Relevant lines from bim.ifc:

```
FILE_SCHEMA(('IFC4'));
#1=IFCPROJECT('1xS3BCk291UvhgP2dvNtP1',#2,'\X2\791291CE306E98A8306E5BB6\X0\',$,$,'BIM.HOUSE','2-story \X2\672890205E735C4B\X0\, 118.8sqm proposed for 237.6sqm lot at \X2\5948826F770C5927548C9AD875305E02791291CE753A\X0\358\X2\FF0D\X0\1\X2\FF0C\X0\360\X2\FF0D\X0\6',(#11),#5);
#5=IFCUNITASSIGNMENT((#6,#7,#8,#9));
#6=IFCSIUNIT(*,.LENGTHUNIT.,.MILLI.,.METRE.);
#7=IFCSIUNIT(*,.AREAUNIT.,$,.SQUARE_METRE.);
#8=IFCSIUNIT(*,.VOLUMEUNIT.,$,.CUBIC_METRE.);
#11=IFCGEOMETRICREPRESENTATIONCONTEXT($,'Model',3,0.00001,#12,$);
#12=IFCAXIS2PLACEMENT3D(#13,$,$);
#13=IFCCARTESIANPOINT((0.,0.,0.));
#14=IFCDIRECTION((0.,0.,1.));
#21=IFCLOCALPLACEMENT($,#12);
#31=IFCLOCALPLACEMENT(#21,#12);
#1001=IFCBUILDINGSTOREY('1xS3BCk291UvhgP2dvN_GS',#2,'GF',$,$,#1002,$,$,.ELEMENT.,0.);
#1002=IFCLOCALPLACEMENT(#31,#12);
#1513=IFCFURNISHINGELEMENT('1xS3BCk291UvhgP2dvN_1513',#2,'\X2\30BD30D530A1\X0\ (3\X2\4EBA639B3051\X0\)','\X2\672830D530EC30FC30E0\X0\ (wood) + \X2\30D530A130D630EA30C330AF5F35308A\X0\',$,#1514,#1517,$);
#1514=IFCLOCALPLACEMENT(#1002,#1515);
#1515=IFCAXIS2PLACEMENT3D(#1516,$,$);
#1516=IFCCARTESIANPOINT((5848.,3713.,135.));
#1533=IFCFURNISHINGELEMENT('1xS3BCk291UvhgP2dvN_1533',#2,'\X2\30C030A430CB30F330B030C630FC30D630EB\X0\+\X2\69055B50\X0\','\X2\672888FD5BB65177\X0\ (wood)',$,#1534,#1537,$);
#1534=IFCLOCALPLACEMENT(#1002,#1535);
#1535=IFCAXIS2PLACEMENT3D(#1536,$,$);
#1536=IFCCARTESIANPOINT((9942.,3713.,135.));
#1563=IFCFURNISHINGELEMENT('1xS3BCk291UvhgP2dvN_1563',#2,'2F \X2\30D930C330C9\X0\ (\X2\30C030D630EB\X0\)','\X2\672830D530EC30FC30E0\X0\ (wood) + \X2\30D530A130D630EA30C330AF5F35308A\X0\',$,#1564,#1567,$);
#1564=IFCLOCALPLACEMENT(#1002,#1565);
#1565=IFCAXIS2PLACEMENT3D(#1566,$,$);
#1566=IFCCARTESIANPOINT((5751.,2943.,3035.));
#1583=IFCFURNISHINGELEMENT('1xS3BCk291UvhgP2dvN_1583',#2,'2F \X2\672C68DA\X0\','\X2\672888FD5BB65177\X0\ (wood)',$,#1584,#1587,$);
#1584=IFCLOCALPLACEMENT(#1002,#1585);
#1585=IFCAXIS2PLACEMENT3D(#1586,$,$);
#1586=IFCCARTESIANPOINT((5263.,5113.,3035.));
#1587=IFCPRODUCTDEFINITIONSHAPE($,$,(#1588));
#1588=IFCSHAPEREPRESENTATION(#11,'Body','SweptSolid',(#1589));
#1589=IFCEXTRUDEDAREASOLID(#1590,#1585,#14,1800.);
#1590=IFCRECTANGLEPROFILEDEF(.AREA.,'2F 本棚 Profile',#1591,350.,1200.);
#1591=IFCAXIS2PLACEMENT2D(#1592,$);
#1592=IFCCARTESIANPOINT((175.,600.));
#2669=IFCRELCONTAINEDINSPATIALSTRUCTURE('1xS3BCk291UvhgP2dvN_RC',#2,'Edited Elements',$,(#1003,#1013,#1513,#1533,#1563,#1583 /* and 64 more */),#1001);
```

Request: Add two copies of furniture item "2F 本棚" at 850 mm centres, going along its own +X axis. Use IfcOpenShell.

```python
import ifcopenshell
import ifcopenshell.api.geometry
import ifcopenshell.api.root
import ifcopenshell.util.element
import ifcopenshell.util.placement
import ifcopenshell.util.unit

model = ifcopenshell.open("bim.ifc")
unit_scale = ifcopenshell.util.unit.calculate_unit_scale(model)


def reuse_history(source, copy):
    """copy_class also copies each property set's owner history, people and application; keep the originals."""
    for rel in copy.IsDefinedBy:
        if rel.is_a("IfcRelDefinesByProperties") and (history := rel.RelatingPropertyDefinition.OwnerHistory):
            rel.RelatingPropertyDefinition.OwnerHistory = source.OwnerHistory
            ifcopenshell.util.element.remove_deep2(model, history)


source = model.by_guid("1xS3BCk291UvhgP2dvN_1583")
base = ifcopenshell.util.placement.get_local_placement(source.ObjectPlacement)
step = base[:3, 0] * 0.85 / unit_scale

for i in range(1, 3):
    copy = ifcopenshell.api.root.copy_class(model, product=source)
    copy.Representation = ifcopenshell.util.element.copy_deep(
        model, source.Representation, exclude=["IfcGeometricRepresentationContext", "IfcRepresentationMap"]
    )
    reuse_history(source, copy)
    matrix = base.copy()
    matrix[:3, 3] += i * step
    print("added at", matrix[:3, 3].round(3) + 0.0)
    ifcopenshell.api.geometry.edit_object_placement(model, product=copy, matrix=matrix, is_si=False)

model.write("bim-out.ifc")
```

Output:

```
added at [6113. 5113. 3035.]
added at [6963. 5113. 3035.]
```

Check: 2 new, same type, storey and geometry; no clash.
